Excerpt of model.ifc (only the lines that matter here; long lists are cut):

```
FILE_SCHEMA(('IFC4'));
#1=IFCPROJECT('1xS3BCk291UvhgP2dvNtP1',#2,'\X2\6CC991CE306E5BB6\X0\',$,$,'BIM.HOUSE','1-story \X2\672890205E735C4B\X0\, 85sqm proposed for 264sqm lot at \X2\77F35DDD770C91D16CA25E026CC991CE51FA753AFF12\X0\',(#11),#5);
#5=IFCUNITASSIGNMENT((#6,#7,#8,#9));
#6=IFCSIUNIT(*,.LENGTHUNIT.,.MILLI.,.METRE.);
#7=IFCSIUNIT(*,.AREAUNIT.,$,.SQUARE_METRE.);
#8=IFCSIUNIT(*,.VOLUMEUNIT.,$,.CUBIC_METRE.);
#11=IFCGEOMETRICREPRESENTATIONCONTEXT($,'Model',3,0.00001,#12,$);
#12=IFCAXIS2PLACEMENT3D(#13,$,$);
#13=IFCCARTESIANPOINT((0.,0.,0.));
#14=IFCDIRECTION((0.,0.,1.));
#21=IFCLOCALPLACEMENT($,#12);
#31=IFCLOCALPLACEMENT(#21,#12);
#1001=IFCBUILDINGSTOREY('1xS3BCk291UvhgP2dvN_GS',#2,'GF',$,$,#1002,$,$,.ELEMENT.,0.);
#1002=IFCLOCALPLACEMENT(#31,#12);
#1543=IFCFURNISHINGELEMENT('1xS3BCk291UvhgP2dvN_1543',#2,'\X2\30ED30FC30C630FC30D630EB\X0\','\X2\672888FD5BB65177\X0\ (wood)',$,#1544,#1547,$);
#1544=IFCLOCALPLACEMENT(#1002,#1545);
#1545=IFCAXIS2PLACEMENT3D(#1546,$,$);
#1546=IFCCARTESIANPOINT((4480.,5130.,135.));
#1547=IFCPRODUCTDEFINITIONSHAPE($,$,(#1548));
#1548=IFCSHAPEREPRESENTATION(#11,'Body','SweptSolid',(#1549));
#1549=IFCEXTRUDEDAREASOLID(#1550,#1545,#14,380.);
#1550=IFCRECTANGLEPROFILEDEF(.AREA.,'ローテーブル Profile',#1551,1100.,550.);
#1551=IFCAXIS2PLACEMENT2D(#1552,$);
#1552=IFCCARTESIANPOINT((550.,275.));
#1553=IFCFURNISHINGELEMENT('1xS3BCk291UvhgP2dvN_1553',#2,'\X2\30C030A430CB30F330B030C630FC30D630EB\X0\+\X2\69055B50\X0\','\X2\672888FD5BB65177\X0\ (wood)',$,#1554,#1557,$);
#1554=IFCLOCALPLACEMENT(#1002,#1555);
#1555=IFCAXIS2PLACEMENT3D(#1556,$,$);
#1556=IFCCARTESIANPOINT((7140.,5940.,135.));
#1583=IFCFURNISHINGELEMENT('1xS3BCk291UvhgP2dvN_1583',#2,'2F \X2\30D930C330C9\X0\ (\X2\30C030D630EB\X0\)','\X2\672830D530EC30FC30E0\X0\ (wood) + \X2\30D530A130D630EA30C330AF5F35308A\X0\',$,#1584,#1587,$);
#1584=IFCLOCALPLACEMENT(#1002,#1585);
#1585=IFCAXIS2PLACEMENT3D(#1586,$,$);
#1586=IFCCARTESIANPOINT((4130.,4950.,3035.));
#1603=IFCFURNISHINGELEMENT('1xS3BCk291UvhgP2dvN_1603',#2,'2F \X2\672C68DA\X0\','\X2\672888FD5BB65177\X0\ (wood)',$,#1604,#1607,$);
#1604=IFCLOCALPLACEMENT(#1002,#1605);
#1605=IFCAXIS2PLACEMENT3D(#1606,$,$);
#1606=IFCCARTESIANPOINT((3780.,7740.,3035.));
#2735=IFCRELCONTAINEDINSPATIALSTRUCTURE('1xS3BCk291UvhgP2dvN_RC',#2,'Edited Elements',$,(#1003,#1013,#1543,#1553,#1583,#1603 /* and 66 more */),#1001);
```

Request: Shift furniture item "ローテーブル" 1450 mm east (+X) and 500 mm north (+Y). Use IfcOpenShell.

```python
import ifcopenshell
import ifcopenshell.api.geometry
import ifcopenshell.util.placement
import ifcopenshell.util.unit

model = ifcopenshell.open("model.ifc")
unit_scale = ifcopenshell.util.unit.calculate_unit_scale(model)

item = model.by_guid("1xS3BCk291UvhgP2dvN_1543")
matrix = ifcopenshell.util.placement.get_local_placement(item.ObjectPlacement)
matrix[0, 3] += 1.45 / unit_scale
matrix[1, 3] += 0.5 / unit_scale
ifcopenshell.api.geometry.edit_object_placement(model, product=item, matrix=matrix, is_si=False)

print(ifcopenshell.util.placement.get_local_placement(item.ObjectPlacement).round(3) + 0.0)

model.write("model_v2.ifc")
```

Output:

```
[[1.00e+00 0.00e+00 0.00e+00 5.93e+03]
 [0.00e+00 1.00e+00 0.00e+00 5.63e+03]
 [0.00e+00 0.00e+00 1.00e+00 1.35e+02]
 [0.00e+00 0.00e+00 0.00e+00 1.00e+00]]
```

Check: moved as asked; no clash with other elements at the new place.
